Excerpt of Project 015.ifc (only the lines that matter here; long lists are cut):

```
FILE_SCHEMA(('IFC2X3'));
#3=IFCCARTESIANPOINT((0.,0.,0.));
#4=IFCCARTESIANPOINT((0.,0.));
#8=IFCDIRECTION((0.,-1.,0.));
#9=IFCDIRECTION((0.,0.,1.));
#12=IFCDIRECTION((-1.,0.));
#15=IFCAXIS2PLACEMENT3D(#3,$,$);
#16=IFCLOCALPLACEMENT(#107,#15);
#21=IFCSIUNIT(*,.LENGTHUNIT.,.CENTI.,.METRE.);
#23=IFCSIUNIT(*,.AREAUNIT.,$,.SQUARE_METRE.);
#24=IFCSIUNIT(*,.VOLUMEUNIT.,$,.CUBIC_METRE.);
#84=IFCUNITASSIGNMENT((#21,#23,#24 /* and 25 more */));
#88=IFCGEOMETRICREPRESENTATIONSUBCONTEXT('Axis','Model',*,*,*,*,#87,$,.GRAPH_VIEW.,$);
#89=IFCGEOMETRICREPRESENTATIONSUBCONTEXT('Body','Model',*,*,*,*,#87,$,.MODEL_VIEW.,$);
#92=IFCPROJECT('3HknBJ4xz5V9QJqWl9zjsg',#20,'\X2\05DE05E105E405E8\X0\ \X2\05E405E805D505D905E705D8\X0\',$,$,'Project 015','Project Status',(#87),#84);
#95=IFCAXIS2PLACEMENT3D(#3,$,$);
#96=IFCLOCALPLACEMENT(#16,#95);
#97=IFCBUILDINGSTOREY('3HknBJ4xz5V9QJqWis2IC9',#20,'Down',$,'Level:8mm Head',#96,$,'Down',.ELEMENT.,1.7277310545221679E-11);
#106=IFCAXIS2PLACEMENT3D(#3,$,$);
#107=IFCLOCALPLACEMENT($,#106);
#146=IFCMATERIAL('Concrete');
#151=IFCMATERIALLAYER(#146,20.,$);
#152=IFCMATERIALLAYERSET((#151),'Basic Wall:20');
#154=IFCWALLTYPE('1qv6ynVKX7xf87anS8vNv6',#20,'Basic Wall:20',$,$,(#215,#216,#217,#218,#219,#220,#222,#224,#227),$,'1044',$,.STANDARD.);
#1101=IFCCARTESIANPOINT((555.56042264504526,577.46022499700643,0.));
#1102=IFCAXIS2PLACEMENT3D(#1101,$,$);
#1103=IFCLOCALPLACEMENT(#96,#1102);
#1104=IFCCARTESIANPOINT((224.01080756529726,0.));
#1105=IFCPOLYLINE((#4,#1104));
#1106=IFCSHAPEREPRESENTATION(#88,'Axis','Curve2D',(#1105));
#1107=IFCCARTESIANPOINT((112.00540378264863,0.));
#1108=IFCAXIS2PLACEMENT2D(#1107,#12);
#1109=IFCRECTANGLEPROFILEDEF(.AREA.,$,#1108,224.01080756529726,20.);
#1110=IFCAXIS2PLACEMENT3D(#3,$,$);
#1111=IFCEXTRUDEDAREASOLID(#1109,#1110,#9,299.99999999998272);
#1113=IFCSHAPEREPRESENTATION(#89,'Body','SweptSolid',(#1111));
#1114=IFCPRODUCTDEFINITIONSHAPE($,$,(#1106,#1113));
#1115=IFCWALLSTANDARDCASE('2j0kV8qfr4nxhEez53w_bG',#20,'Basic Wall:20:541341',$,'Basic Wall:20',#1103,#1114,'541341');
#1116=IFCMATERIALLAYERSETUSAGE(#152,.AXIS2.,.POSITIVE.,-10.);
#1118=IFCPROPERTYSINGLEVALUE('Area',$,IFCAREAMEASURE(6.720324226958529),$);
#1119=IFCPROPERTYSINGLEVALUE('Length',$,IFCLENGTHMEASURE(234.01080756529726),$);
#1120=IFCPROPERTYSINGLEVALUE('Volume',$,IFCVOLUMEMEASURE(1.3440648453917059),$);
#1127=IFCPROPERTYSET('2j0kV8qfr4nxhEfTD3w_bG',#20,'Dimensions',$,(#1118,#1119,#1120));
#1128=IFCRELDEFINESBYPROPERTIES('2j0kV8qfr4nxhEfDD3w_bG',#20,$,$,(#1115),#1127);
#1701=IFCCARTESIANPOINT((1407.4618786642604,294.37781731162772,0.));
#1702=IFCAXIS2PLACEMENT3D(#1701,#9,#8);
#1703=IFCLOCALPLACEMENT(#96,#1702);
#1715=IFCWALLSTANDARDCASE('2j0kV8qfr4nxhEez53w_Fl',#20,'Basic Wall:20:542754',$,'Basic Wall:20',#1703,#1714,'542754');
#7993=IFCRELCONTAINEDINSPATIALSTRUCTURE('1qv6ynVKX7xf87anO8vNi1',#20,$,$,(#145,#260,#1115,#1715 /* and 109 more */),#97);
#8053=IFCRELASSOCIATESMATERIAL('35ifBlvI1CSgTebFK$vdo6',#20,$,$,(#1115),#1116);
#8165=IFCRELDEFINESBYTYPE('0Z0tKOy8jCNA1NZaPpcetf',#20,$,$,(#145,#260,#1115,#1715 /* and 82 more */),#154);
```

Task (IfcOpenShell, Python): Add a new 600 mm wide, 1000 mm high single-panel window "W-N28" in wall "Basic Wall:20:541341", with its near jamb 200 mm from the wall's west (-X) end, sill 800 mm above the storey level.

```python
import numpy as np
import ifcopenshell
import ifcopenshell.api.feature
import ifcopenshell.api.geometry
import ifcopenshell.api.pset
import ifcopenshell.api.root
import ifcopenshell.api.spatial
import ifcopenshell.api.type
import ifcopenshell.geom
import ifcopenshell.util.element
import ifcopenshell.util.placement
import ifcopenshell.util.representation
import ifcopenshell.util.shape
import ifcopenshell.util.unit

model = ifcopenshell.open("Project 015.ifc")
unit_scale = ifcopenshell.util.unit.calculate_unit_scale(model)
area_scale = ifcopenshell.util.unit.calculate_unit_scale(model, "AREAUNIT")
volume_scale = ifcopenshell.util.unit.calculate_unit_scale(model, "VOLUMEUNIT")
settings = ifcopenshell.geom.settings()


def volume(element):
    """Net volume in cubic metres, openings subtracted."""
    shape = ifcopenshell.geom.create_shape(settings, element)
    return ifcopenshell.util.shape.get_volume(shape.geometry)


wall = model.by_id(1115)
storey = ifcopenshell.util.element.get_container(wall, ifc_class="IfcBuildingStorey")
context = ifcopenshell.util.representation.get_context(model, "Model", "Body", "MODEL_VIEW")
before = volume(wall)

width, height, from_end, sill = 0.6, 1, 0.2, 0.8  # metres

# The wall runs along its own X axis, and the end named is its -X end.
wall_shape = ifcopenshell.geom.create_shape(settings, wall)
x, y, z = ifcopenshell.util.shape.get_vertices(wall_shape.geometry).T
start = x.min() + from_end
face, thickness = float(y.min()), float(y.max() - y.min())
wall_matrix = ifcopenshell.util.placement.get_local_placement(wall.ObjectPlacement)
level = ifcopenshell.util.placement.get_local_placement(storey.ObjectPlacement)[2, 3]


def in_wall(x, y):
    """Placement at x, y metres in the wall's axes, at sill height."""
    matrix = wall_matrix.copy()
    matrix[:, 3] = wall_matrix @ np.array([x / unit_scale, y / unit_scale, 0.0, 1.0])
    matrix[2, 3] = level + sill / unit_scale
    return matrix


# Opening: a box that overshoots both wall faces by 50 mm.
opening = ifcopenshell.api.root.create_entity(model, ifc_class="IfcOpeningElement")
box = ifcopenshell.api.geometry.add_wall_representation(
    model, context=context, length=width, height=height, thickness=thickness + 0.1
)
ifcopenshell.api.geometry.assign_representation(model, product=opening, representation=box)
ifcopenshell.api.geometry.edit_object_placement(model, product=opening, matrix=in_wall(start, face - 0.05), is_si=False)
ifcopenshell.api.feature.add_feature(model, feature=opening, element=wall)

window = ifcopenshell.api.root.create_entity(model, ifc_class="IfcWindow", name="W-N28")
window.OverallWidth, window.OverallHeight = width / unit_scale, height / unit_scale
body = ifcopenshell.api.geometry.add_window_representation(
    model,
    context=context,
    overall_width=window.OverallWidth,
    overall_height=window.OverallHeight,
    partition_type="SINGLE_PANEL",
)
ifcopenshell.api.geometry.assign_representation(model, product=window, representation=body)
ifcopenshell.api.spatial.assign_container(model, products=[window], relating_structure=storey)
fills = ifcopenshell.api.feature.add_filling(model, opening=opening, element=window)
fills.OwnerHistory = window.OwnerHistory  # required in IFC2X3

# IFC2X3 keeps the operation on the window style.
style = ifcopenshell.api.root.create_entity(model, ifc_class="IfcWindowStyle", name="W-N28")
style.OperationType, style.ConstructionType = "SINGLE_PANEL", "NOTDEFINED"
style.ParameterTakesPrecedence = style.Sizeable = False
ifcopenshell.api.type.assign_type(model, related_objects=[window], relating_type=style)

# Centre the window in the wall's thickness.
ifcopenshell.api.geometry.edit_object_placement(model, product=window, matrix=in_wall(start, face), is_si=False)
window_shape = ifcopenshell.geom.create_shape(settings, window)
depth = ifcopenshell.util.shape.get_vertices(window_shape.geometry)[:, 1]
offset = face + thickness / 2 - (depth.min() + depth.max()) / 2
ifcopenshell.api.geometry.edit_object_placement(model, product=window, matrix=in_wall(start, offset), is_si=False)

after = volume(wall)

# Update the wall's stored quantities.
pset = model.by_id(ifcopenshell.util.element.get_pset(wall, "Dimensions", should_inherit=False)["id"])
ifcopenshell.api.pset.edit_pset(model, pset=pset, properties={
    "Area": model.create_entity("IfcAreaMeasure", after / thickness / area_scale),
    "Volume": model.create_entity("IfcVolumeMeasure", after / volume_scale),
})

print(f"wall volume {before:.3f} -> {after:.3f} m3")

model.write("Project 015_edited.ifc")
```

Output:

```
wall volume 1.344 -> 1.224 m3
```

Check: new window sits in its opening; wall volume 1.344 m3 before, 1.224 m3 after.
